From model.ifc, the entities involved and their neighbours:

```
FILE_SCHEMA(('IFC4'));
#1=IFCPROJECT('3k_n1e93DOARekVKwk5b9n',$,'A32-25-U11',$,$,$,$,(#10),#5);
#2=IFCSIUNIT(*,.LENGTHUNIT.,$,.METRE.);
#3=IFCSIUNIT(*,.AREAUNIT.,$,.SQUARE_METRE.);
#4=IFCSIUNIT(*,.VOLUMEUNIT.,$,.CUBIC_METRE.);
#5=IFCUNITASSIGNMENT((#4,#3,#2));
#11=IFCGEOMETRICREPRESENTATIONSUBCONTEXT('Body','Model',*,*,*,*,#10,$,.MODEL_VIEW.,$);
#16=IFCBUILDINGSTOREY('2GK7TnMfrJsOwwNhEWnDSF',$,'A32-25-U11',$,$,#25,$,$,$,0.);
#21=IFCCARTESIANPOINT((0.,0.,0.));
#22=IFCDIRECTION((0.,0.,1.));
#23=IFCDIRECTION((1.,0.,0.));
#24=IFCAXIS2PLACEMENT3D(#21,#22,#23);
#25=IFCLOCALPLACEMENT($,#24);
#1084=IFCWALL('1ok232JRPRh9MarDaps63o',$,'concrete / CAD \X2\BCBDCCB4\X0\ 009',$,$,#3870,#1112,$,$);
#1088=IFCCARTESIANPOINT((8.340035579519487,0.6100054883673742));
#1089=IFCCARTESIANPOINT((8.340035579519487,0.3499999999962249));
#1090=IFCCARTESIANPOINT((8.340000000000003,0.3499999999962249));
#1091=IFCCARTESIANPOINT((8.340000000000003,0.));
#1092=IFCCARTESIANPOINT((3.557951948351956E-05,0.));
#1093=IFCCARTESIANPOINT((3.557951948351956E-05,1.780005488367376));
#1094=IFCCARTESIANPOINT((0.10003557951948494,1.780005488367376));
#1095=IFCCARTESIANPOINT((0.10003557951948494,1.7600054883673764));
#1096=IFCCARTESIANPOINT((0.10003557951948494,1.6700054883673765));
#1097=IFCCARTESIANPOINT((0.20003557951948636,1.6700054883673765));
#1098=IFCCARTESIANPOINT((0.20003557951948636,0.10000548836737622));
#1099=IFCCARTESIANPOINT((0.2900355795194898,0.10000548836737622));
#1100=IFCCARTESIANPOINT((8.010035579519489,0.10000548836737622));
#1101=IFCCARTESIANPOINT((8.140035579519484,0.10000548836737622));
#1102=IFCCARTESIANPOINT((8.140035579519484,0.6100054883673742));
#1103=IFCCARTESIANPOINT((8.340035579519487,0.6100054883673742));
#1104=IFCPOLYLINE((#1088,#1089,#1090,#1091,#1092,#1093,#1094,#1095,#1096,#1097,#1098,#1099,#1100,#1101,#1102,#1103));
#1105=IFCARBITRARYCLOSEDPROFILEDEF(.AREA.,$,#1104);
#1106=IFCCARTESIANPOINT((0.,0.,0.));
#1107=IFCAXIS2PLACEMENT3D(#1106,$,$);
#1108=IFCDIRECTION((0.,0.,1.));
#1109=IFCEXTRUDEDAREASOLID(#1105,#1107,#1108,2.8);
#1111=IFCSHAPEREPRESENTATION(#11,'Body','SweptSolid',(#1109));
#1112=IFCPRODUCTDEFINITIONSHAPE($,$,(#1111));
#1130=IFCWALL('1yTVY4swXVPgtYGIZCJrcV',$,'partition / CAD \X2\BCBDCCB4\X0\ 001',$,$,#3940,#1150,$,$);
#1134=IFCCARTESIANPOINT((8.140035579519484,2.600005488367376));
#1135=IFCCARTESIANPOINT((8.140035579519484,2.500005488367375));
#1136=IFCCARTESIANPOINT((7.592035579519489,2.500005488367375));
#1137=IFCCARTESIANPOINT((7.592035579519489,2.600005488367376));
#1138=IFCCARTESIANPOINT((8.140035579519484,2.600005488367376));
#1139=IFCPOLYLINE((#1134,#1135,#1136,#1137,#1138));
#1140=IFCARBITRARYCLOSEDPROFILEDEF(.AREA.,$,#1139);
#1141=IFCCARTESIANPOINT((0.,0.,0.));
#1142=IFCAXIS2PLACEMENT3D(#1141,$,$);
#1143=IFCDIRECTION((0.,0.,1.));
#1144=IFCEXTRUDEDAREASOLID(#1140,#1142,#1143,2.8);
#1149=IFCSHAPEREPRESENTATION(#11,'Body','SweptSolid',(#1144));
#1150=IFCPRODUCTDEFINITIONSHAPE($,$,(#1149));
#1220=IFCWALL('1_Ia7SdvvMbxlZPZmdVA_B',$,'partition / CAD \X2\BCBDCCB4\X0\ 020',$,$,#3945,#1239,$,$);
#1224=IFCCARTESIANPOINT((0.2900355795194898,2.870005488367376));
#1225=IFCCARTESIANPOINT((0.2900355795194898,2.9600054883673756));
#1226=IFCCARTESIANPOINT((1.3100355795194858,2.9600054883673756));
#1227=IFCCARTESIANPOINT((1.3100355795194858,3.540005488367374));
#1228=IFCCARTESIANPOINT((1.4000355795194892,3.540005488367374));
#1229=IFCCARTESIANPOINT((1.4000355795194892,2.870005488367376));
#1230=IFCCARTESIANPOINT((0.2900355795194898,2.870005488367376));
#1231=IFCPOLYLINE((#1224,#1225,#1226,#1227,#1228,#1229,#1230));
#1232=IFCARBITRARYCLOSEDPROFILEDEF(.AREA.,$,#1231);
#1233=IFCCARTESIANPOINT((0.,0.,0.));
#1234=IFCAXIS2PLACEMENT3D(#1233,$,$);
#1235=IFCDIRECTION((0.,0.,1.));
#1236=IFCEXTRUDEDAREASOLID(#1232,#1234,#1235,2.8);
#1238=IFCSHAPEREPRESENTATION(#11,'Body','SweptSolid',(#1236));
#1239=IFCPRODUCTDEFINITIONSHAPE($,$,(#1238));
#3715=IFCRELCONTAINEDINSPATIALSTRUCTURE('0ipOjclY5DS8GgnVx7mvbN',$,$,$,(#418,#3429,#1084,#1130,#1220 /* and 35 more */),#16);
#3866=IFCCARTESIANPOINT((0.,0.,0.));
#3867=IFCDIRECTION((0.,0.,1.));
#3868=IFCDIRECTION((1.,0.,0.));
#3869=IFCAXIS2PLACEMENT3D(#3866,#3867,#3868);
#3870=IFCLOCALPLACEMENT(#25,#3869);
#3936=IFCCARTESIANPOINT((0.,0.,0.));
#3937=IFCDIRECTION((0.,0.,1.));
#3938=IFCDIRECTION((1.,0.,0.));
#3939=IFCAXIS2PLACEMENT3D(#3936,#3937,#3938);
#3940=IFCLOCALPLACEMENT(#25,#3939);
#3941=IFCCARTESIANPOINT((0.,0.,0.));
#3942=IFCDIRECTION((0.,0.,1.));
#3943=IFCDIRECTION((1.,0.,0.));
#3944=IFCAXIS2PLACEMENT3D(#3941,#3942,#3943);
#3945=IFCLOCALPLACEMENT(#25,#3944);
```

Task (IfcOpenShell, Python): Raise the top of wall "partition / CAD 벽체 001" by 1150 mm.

```python
import ifcopenshell
import ifcopenshell.geom
import ifcopenshell.util.representation
import ifcopenshell.util.shape

model = ifcopenshell.open("model.ifc")
settings = ifcopenshell.geom.settings()


def volume(element):
    """Net volume in cubic metres, openings subtracted."""
    shape = ifcopenshell.geom.create_shape(settings, element)
    return ifcopenshell.util.shape.get_volume(shape.geometry)


wall = model.by_guid("1yTVY4swXVPgtYGIZCJrcV")
before = volume(wall)

body = ifcopenshell.util.representation.get_representation(wall, "Model", "Body")
solid = body.Items[0]
old_height = solid.Depth
solid.Depth += 1.15
after = volume(wall)

print(f"height {old_height:g} -> {solid.Depth:g}, volume {before:.3f} -> {after:.3f} m3")

model.write("model-out.ifc")
```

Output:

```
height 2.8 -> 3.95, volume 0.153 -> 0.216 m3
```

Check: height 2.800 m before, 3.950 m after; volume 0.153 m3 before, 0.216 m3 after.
